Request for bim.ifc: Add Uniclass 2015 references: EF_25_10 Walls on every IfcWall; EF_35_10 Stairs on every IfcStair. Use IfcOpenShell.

First a look at what the model holds.

```python
import ifcopenshell

model = ifcopenshell.open("bim.ifc")
print(model.schema)
print("classifications:", [c.Name for c in model.by_type("IfcClassification")])
for ifc_class in ("IfcDoor", "IfcRoof", "IfcStair", "IfcWall", "IfcWindow"):
    print(ifc_class, len(model.by_type(ifc_class)))
```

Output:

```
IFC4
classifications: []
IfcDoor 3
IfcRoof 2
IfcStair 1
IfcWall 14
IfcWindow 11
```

```python
import ifcopenshell
import ifcopenshell.api.classification

model = ifcopenshell.open("bim.ifc")

system = ifcopenshell.api.classification.add_classification(model, classification="Uniclass 2015")

codes = {
    "IfcWall": ("EF_25_10", "Walls"),
    "IfcStair": ("EF_35_10", "Stairs"),
}
for ifc_class, (code, name) in codes.items():
    products = model.by_type(ifc_class)
    ifcopenshell.api.classification.add_reference(
        model, products=products, classification=system, identification=code, name=name
    )
    print(code, len(products))

model.write("bim-out.ifc")
```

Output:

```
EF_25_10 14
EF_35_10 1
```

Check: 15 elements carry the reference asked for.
